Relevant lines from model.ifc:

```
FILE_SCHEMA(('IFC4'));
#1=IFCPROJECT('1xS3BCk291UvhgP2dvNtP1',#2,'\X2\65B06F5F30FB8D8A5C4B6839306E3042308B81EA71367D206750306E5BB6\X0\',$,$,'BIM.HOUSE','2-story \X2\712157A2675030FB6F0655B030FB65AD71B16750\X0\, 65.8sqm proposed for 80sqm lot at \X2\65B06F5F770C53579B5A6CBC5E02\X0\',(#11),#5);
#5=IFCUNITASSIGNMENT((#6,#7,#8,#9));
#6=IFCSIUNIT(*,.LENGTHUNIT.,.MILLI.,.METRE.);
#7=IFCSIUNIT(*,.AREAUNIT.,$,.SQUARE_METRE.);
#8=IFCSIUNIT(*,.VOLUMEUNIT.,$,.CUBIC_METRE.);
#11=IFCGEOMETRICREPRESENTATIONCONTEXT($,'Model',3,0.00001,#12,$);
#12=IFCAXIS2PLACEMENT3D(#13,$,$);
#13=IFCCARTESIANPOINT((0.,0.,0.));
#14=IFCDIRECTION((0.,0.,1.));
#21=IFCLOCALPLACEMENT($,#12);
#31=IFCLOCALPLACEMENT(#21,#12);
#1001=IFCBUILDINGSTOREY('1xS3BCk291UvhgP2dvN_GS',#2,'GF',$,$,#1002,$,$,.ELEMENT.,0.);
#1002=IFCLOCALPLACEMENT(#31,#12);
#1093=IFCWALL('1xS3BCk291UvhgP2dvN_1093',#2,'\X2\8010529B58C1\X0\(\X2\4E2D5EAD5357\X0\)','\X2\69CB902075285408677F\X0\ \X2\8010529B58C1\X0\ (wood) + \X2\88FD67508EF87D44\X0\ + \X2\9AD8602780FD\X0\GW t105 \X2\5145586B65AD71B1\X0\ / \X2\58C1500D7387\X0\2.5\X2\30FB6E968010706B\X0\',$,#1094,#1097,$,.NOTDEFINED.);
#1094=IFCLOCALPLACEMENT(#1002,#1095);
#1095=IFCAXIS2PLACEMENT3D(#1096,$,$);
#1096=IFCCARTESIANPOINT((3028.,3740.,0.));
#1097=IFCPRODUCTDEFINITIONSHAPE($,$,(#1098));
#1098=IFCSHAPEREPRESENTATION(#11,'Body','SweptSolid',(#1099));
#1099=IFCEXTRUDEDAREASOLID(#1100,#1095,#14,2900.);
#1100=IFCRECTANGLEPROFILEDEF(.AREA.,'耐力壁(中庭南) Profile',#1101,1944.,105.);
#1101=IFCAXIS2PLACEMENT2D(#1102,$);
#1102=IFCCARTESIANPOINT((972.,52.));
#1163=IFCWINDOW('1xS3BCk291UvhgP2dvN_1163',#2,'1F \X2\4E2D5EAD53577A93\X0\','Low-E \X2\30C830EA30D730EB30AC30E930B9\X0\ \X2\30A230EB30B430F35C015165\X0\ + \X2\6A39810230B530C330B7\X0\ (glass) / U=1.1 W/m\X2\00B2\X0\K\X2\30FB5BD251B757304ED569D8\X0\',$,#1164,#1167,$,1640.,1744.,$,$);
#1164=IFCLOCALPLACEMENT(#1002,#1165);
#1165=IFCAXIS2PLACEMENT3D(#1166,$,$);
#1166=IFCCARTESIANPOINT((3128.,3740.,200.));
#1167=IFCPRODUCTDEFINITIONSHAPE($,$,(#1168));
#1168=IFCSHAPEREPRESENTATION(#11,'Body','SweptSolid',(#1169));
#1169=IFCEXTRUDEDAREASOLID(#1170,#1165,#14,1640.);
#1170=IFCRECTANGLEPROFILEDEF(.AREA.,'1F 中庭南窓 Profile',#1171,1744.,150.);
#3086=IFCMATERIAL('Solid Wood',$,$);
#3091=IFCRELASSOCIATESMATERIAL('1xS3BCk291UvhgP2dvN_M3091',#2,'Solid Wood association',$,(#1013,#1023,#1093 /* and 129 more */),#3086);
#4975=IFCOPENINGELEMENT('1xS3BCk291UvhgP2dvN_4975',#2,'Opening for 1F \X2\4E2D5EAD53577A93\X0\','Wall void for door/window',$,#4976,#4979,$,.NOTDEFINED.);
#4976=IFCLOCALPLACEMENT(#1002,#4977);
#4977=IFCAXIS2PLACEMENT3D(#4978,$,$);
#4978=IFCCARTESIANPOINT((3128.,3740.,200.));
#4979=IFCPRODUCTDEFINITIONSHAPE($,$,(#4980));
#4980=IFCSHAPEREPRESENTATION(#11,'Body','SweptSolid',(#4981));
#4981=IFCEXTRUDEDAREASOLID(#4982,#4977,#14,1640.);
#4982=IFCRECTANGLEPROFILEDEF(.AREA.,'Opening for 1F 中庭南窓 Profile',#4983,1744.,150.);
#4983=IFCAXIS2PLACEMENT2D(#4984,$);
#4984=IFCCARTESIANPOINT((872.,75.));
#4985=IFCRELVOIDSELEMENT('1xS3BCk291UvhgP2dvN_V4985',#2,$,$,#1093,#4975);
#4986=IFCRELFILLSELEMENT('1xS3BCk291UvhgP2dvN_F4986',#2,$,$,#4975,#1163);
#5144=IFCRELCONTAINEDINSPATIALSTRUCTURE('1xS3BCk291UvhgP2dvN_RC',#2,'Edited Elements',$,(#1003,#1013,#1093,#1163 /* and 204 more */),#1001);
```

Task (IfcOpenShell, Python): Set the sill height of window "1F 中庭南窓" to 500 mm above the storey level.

```python
import numpy as np
import ifcopenshell
import ifcopenshell.api.geometry
import ifcopenshell.geom
import ifcopenshell.util.element
import ifcopenshell.util.placement
import ifcopenshell.util.shape
import ifcopenshell.util.unit

model = ifcopenshell.open("model.ifc")
unit_scale = ifcopenshell.util.unit.calculate_unit_scale(model)

window = model.by_guid("1xS3BCk291UvhgP2dvN_1163")
opening = window.FillsVoids[0].RelatingOpeningElement
storey = ifcopenshell.util.element.get_container(window, ifc_class="IfcBuildingStorey")
level = ifcopenshell.util.placement.get_local_placement(storey.ObjectPlacement)[2, 3]

# The opening's origin need not be at the sill, so measure its lowest point.
shape = ifcopenshell.geom.create_shape(ifcopenshell.geom.settings(), opening)
bottom = ifcopenshell.util.shape.get_shape_bottom_elevation(shape, shape.geometry) / unit_scale
dz = level + 500.0 - bottom

shift = np.array([0.0, 0.0, dz])
# The window is not placed relative to its opening, so move both.
for product in (opening, window):
    matrix = ifcopenshell.util.placement.get_local_placement(product.ObjectPlacement)
    matrix[:3, 3] += shift
    ifcopenshell.api.geometry.edit_object_placement(model, product=product, matrix=matrix, is_si=False)

print(f"moved by {dz * unit_scale:+.3f} m")

model.write("model_v2.ifc")
```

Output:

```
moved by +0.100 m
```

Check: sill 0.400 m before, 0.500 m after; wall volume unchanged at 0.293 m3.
